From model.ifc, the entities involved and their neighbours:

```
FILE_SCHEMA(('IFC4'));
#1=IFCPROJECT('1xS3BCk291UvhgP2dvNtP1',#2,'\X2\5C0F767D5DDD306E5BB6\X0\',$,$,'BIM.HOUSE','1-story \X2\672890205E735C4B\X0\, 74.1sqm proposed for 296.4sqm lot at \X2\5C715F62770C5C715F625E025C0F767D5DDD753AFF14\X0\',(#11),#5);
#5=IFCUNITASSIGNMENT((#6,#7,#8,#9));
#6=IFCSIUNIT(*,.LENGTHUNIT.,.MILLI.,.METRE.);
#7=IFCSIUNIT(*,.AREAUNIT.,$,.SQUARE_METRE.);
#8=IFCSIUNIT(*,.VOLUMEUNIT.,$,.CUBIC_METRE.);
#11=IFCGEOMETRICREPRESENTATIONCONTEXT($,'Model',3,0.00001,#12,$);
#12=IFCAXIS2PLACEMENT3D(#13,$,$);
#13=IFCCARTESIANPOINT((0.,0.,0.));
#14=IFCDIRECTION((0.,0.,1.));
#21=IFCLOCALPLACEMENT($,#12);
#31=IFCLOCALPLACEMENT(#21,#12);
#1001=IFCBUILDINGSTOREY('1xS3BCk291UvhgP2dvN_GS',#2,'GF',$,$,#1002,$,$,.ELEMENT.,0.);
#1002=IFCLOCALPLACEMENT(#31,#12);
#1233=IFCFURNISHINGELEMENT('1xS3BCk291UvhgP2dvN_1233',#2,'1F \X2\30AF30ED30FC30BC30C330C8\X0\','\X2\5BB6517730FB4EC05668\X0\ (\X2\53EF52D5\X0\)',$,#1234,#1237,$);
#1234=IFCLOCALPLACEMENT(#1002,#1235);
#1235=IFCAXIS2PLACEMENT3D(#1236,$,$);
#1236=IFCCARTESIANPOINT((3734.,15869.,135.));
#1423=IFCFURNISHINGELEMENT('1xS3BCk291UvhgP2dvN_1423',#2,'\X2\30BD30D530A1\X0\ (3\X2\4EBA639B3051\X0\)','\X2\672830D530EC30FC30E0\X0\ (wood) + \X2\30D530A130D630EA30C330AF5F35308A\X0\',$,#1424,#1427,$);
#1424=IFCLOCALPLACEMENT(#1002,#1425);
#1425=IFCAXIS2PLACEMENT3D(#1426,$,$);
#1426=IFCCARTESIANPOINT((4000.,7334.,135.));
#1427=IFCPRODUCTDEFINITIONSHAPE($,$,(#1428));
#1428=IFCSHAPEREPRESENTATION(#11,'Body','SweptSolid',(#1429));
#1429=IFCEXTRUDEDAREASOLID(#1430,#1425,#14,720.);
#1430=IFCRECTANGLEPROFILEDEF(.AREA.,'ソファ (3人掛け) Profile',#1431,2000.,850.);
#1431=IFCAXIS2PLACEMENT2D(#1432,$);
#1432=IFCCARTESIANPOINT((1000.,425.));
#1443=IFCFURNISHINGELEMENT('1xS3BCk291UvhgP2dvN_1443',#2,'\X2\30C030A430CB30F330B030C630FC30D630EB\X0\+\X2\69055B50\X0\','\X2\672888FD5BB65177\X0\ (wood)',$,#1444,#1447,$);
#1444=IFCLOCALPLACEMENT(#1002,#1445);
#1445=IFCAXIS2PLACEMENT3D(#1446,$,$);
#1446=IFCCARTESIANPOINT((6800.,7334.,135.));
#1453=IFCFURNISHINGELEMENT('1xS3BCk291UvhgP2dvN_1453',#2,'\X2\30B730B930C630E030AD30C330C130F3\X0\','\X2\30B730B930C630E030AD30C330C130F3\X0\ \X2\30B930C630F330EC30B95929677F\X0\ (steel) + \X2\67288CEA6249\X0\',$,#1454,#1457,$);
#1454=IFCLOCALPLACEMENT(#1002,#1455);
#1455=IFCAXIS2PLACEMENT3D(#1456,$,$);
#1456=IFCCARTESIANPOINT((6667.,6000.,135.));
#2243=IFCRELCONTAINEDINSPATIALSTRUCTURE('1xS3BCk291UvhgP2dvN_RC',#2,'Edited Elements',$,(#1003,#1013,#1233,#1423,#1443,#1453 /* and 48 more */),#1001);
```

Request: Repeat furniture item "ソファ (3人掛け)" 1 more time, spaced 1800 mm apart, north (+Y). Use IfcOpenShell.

```python
import numpy as np
import ifcopenshell
import ifcopenshell.api.geometry
import ifcopenshell.api.root
import ifcopenshell.util.element
import ifcopenshell.util.placement

model = ifcopenshell.open("model.ifc")


def reuse_history(source, copy):
    """copy_class also copies each property set's owner history, people and application; keep the originals."""
    for rel in copy.IsDefinedBy:
        if rel.is_a("IfcRelDefinesByProperties") and (history := rel.RelatingPropertyDefinition.OwnerHistory):
            rel.RelatingPropertyDefinition.OwnerHistory = source.OwnerHistory
            ifcopenshell.util.element.remove_deep2(model, history)


source = model.by_guid("1xS3BCk291UvhgP2dvN_1423")
base = ifcopenshell.util.placement.get_local_placement(source.ObjectPlacement)
step = np.array([0.0, 1.0, 0.0]) * 1800.0

for i in range(1, 2):
    copy = ifcopenshell.api.root.copy_class(model, product=source)
    copy.Representation = ifcopenshell.util.element.copy_deep(
        model, source.Representation, exclude=["IfcGeometricRepresentationContext", "IfcRepresentationMap"]
    )
    reuse_history(source, copy)
    matrix = base.copy()
    matrix[:3, 3] += i * step
    print("added at", matrix[:3, 3].round(3) + 0.0)
    ifcopenshell.api.geometry.edit_object_placement(model, product=copy, matrix=matrix, is_si=False)

model.write("model_edited.ifc")
```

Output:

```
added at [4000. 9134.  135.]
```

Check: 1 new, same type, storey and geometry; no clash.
